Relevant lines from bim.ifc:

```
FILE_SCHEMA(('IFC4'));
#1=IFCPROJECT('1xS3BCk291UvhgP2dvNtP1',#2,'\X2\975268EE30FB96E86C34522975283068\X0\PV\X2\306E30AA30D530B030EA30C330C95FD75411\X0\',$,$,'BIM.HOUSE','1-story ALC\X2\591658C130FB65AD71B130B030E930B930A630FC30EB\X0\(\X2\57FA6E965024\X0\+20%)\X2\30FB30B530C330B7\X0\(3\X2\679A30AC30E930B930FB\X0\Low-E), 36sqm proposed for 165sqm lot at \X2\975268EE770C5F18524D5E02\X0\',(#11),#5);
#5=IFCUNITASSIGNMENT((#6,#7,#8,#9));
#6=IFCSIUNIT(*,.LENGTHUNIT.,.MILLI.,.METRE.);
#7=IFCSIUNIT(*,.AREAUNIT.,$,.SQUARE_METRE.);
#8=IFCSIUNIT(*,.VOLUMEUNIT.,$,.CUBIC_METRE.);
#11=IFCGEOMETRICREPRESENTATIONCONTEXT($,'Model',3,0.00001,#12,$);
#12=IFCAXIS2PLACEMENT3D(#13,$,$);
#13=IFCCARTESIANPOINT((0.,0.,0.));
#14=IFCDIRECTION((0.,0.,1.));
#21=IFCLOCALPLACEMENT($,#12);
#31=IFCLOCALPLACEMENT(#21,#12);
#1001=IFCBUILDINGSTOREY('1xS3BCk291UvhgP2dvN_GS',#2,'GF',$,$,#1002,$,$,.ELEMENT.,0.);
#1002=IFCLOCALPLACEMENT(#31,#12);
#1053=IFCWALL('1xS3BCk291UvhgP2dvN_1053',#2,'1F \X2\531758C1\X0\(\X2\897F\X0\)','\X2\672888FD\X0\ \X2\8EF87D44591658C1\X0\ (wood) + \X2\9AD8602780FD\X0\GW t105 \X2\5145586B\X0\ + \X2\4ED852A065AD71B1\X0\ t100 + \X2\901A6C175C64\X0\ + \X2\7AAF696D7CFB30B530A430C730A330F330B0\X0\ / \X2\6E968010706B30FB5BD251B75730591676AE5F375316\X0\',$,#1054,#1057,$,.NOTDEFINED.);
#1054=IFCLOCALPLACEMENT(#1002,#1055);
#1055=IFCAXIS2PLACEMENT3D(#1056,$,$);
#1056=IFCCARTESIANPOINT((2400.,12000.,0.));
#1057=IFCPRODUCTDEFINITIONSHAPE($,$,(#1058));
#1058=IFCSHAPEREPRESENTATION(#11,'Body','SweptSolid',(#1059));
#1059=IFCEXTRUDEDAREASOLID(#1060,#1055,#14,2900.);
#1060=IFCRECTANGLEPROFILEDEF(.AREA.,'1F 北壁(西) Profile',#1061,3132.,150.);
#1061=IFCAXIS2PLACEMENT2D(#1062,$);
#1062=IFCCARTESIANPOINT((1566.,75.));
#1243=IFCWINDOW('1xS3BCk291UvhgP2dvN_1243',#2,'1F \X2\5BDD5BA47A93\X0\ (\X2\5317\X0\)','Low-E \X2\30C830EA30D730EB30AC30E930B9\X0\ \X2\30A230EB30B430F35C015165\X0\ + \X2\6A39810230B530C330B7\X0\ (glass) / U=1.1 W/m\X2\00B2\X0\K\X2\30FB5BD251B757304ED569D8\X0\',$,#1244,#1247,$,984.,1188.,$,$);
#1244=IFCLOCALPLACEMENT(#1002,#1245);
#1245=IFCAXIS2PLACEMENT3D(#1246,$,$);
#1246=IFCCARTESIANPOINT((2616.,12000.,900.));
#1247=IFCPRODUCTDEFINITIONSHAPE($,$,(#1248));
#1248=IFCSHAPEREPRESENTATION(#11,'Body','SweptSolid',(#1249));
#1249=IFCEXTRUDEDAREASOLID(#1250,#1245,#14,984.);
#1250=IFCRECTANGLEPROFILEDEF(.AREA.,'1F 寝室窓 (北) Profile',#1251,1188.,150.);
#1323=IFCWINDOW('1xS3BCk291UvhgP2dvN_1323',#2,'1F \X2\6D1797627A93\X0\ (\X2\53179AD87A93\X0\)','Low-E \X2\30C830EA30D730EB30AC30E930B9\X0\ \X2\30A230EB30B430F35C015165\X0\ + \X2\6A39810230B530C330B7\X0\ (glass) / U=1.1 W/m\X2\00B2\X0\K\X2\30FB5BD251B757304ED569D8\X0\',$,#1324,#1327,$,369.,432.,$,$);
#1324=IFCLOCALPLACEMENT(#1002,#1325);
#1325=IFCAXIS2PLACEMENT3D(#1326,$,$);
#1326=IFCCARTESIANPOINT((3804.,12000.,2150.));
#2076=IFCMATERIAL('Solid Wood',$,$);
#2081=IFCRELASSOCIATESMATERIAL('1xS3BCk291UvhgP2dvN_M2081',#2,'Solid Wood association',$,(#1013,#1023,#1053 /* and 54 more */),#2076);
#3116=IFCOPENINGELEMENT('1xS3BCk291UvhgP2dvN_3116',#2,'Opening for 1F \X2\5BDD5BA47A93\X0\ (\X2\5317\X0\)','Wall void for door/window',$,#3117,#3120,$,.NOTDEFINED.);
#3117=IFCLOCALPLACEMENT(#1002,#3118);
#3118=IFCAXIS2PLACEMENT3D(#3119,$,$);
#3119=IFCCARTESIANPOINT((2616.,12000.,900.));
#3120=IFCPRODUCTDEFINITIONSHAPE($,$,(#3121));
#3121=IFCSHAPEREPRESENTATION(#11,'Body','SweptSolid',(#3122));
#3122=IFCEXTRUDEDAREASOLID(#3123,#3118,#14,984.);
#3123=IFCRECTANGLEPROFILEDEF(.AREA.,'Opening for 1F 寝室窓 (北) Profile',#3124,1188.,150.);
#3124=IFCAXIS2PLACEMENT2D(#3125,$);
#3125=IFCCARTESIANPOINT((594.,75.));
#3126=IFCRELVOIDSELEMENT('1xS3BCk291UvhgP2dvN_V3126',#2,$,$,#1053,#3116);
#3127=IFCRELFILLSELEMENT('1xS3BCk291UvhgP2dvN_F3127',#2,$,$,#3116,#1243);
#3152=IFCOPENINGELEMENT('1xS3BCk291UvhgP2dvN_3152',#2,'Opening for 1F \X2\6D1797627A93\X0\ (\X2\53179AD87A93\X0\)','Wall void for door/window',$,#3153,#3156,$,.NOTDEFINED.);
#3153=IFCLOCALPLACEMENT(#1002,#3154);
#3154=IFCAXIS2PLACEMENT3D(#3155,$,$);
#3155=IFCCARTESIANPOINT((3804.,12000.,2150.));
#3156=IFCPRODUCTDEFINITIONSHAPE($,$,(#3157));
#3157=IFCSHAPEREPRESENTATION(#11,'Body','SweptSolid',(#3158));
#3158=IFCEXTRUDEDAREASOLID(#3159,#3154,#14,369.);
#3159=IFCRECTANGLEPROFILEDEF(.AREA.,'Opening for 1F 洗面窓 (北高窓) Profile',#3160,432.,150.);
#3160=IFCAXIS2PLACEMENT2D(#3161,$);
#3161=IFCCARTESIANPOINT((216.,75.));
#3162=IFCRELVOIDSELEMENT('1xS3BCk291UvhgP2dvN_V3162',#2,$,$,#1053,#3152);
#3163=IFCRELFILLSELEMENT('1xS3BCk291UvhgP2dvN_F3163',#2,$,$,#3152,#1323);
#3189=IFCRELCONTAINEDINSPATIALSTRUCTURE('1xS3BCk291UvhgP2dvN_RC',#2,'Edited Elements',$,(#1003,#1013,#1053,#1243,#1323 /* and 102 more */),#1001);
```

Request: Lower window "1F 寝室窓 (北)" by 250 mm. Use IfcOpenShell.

```python
import numpy as np
import ifcopenshell
import ifcopenshell.api.geometry
import ifcopenshell.util.placement
import ifcopenshell.util.unit

model = ifcopenshell.open("bim.ifc")
unit_scale = ifcopenshell.util.unit.calculate_unit_scale(model)

window = model.by_id(1243)
opening = window.FillsVoids[0].RelatingOpeningElement
dz = -250.0

shift = np.array([0.0, 0.0, dz])
# The window is not placed relative to its opening, so move both.
for product in (opening, window):
    matrix = ifcopenshell.util.placement.get_local_placement(product.ObjectPlacement)
    matrix[:3, 3] += shift
    ifcopenshell.api.geometry.edit_object_placement(model, product=product, matrix=matrix, is_si=False)

print(f"moved by {dz * unit_scale:+.3f} m")

model.write("bim_v2.ifc")
```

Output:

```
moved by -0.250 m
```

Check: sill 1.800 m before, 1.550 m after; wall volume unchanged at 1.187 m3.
